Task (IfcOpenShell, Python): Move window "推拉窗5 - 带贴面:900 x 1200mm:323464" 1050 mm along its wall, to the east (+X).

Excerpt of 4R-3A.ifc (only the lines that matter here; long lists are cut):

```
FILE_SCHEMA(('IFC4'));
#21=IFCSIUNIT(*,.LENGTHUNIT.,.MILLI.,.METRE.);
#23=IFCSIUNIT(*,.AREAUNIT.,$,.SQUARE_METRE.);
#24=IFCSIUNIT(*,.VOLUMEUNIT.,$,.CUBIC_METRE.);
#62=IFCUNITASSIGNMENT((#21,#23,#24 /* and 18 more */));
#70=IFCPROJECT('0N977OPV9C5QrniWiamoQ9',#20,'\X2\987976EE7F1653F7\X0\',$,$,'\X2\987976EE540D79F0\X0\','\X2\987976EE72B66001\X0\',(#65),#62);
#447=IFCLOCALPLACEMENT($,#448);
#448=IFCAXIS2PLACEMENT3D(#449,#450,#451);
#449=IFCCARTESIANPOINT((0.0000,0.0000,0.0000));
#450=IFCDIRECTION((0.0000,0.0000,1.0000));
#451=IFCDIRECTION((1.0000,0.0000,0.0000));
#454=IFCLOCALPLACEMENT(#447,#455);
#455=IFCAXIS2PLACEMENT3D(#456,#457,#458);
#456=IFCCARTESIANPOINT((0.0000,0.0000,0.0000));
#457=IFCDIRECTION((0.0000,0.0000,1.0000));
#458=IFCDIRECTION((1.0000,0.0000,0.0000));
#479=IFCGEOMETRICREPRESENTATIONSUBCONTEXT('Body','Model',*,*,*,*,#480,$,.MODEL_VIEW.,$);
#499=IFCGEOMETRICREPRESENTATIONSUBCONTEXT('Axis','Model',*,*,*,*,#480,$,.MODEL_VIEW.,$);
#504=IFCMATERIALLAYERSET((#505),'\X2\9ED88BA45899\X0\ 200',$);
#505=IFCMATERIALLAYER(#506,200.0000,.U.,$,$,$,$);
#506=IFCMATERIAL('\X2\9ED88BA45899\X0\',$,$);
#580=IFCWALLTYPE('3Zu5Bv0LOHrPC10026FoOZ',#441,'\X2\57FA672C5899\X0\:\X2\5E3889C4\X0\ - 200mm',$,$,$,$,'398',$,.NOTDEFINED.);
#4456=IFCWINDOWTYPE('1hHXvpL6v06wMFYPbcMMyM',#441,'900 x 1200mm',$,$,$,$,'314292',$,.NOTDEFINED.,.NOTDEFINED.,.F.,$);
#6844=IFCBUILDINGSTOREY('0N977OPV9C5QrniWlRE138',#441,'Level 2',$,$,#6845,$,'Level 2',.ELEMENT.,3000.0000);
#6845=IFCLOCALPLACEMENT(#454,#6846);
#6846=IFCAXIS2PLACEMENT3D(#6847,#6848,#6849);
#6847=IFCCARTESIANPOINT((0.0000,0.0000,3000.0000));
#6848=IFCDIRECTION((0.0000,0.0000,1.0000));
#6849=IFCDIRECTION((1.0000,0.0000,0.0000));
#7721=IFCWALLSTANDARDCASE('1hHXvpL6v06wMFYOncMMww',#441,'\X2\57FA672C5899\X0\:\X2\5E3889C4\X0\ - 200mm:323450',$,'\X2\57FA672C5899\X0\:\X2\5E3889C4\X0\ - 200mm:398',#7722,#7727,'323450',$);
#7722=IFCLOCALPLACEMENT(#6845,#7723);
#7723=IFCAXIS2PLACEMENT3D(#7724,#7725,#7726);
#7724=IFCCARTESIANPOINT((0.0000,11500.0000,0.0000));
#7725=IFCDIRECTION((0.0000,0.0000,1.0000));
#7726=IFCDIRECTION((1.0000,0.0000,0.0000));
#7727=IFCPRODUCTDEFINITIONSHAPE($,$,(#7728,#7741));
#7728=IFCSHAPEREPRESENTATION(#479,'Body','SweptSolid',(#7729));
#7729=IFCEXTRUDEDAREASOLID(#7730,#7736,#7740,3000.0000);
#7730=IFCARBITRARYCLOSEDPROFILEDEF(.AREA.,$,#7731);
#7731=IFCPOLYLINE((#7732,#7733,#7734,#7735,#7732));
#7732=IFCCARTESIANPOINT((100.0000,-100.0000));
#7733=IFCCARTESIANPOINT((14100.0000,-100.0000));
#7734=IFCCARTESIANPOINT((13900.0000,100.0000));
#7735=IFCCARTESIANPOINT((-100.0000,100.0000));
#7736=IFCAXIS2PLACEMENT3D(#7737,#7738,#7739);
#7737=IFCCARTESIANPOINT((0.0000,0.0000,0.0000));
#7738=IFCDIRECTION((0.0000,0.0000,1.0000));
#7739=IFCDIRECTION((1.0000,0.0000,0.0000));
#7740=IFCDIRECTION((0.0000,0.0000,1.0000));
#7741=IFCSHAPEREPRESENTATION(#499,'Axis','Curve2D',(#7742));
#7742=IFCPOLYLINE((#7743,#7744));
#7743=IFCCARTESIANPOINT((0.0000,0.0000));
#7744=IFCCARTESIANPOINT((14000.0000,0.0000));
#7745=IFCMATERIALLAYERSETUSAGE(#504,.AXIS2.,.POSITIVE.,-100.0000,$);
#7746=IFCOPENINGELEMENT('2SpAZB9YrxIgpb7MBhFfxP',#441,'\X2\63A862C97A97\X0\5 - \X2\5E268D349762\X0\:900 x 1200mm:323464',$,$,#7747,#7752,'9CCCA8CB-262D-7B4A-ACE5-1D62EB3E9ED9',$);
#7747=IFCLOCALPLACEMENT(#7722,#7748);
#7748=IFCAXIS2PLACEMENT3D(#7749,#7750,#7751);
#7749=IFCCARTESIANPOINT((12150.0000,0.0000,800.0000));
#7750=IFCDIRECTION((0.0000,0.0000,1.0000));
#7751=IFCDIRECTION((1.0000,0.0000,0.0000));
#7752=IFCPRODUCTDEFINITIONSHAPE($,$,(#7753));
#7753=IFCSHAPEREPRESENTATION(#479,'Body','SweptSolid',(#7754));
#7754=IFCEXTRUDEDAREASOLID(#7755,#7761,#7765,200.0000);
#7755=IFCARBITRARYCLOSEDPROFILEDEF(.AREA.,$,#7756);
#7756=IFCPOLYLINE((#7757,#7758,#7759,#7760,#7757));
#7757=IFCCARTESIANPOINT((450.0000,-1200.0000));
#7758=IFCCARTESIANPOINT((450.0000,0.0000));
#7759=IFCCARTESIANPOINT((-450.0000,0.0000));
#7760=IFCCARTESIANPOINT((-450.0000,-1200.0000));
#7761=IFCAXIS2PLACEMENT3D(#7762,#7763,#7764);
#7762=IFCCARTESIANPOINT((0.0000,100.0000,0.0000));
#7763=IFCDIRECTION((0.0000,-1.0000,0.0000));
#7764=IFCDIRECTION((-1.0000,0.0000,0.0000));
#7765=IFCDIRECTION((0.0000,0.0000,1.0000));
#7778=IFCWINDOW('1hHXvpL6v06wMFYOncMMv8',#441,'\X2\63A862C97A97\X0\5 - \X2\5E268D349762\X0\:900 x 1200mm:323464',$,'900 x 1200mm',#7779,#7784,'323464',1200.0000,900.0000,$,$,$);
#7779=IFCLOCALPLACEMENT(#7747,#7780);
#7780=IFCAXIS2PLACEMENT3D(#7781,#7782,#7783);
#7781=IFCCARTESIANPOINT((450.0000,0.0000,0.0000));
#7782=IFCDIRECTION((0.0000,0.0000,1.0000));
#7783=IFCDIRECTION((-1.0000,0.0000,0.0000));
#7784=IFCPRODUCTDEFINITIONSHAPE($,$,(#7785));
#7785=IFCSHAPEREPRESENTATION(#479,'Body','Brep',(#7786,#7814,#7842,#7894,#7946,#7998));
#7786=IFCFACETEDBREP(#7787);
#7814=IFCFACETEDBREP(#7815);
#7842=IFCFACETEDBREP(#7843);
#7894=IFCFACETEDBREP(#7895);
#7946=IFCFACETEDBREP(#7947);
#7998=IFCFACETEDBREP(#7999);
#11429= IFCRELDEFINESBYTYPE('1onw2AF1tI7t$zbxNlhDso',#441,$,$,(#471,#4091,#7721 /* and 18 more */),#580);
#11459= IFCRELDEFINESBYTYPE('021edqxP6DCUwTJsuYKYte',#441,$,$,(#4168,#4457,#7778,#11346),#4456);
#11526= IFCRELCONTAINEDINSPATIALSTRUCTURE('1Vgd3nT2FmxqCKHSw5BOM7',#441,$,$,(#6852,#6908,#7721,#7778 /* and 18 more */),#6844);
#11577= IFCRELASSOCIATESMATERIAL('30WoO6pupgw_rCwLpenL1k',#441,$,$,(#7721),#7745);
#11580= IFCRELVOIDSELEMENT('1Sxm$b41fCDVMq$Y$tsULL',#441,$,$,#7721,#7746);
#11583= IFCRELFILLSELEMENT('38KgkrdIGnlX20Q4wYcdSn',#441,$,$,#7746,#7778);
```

```python
import ifcopenshell
import ifcopenshell.api.geometry
import ifcopenshell.util.placement
import ifcopenshell.util.unit

model = ifcopenshell.open("4R-3A.ifc")
unit_scale = ifcopenshell.util.unit.calculate_unit_scale(model)

window = model.by_guid("1hHXvpL6v06wMFYOncMMv8")
opening = window.FillsVoids[0].RelatingOpeningElement
wall = opening.VoidsElements[0].RelatingBuildingElement

wall_matrix = ifcopenshell.util.placement.get_local_placement(wall.ObjectPlacement)
shift = wall_matrix[:3, 0] * 1.05 / unit_scale
before = ifcopenshell.util.placement.get_local_placement(window.ObjectPlacement)[:3, 3].copy()

# The window is placed relative to its opening, so it follows when the opening moves.
matrix = ifcopenshell.util.placement.get_local_placement(opening.ObjectPlacement)
matrix[:3, 3] += shift
ifcopenshell.api.geometry.edit_object_placement(
    model, product=opening, matrix=matrix, is_si=False, should_transform_children=True
)

after = ifcopenshell.util.placement.get_local_placement(window.ObjectPlacement)[:3, 3]
print("window moved by", (after - before).round(3) + 0.0)

model.write("4R-3A_edited.ifc")
```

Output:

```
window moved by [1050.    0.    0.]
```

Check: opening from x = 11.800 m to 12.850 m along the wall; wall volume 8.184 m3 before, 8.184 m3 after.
